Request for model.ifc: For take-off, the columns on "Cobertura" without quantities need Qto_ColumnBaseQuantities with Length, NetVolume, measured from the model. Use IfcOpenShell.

First a look at what the model holds.

```python
import ifcopenshell
import ifcopenshell.util.element
import ifcopenshell.util.unit

model = ifcopenshell.open("model.ifc")
print(model.schema)
for unit_type in ("LENGTHUNIT", "AREAUNIT", "VOLUMEUNIT"):
    print(unit_type, ifcopenshell.util.unit.calculate_unit_scale(model, unit_type))
storey = next(s for s in model.by_type("IfcBuildingStorey") if s.Name == "Cobertura")
columns = [e for e in ifcopenshell.util.element.get_decomposition(storey) if e.is_a("IfcColumn")]
for e in sorted(columns, key=lambda e: e.id()):
    print(e.id(), e.is_a(), e.Name, list(ifcopenshell.util.element.get_psets(e, qtos_only=True)), sep=" | ")
```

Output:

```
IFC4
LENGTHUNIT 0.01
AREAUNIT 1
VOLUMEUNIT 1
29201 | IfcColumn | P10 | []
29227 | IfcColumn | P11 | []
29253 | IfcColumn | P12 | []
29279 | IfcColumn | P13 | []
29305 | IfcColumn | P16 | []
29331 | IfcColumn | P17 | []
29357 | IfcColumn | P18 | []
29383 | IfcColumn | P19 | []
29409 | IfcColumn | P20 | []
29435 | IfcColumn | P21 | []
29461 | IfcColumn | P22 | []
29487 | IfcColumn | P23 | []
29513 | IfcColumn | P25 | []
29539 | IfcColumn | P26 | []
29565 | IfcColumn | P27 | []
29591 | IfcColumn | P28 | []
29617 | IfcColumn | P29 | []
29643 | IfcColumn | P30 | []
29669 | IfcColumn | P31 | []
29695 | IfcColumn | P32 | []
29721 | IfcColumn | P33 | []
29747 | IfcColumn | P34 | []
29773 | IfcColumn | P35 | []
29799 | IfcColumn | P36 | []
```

```python
import ifcopenshell
import ifcopenshell.api.pset
import ifcopenshell.geom
import ifcopenshell.util.element
import ifcopenshell.util.shape
import ifcopenshell.util.unit

model = ifcopenshell.open("model.ifc")
unit_scale = ifcopenshell.util.unit.calculate_unit_scale(model)
volume_scale = ifcopenshell.util.unit.calculate_unit_scale(model, "VOLUMEUNIT")
settings = ifcopenshell.geom.settings()

storey = next(s for s in model.by_type("IfcBuildingStorey") if s.Name == "Cobertura")
columns = [e for e in ifcopenshell.util.element.get_decomposition(storey) if e.is_a("IfcColumn")]

for e in sorted(columns, key=lambda e: e.id()):
    if ifcopenshell.util.element.get_psets(e, qtos_only=True, should_inherit=False):
        continue
    # Geometry comes back in metres, in the element's own axes.
    shape = ifcopenshell.geom.create_shape(settings, e)
    values = {
        "Length": ifcopenshell.util.shape.get_z(shape.geometry) / unit_scale,
        "NetVolume": ifcopenshell.util.shape.get_volume(shape.geometry) / volume_scale,
    }
    qto = ifcopenshell.api.pset.add_qto(model, product=e, name="Qto_ColumnBaseQuantities")
    ifcopenshell.api.pset.edit_qto(model, qto=qto, properties=values)
    print(e.id(), {k: round(v, 3) for k, v in values.items()})

model.write("model_edited.ifc")
```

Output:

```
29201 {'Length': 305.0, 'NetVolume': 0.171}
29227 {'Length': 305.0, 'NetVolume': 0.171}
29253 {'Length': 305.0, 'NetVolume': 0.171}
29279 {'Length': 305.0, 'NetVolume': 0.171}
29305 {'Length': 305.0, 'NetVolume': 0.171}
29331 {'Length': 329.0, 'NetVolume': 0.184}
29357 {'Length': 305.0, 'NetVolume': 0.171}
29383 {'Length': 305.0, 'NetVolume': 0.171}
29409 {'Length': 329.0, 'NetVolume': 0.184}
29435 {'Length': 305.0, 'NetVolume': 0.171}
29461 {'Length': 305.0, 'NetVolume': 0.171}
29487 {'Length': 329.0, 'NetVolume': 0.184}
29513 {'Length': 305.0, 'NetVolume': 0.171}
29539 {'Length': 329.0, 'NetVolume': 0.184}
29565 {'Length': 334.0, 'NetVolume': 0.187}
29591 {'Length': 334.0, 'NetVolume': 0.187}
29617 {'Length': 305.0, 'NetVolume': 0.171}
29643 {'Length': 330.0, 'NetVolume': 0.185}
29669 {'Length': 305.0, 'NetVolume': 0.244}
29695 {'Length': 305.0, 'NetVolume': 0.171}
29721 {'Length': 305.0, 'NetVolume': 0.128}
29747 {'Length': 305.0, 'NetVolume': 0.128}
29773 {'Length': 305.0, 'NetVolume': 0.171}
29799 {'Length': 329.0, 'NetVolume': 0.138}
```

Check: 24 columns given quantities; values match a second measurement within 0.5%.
